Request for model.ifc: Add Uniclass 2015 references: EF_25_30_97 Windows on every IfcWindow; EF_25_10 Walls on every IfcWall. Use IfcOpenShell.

First a look at what the model holds.

```python
import ifcopenshell

model = ifcopenshell.open("model.ifc")
print(model.schema)
print("classifications:", [c.Name for c in model.by_type("IfcClassification")])
for ifc_class in ("IfcDoor", "IfcRoof", "IfcStair", "IfcWall", "IfcWindow"):
    print(ifc_class, len(model.by_type(ifc_class)))
```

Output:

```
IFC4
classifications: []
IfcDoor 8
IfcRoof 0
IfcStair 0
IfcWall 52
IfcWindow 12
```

```python
import ifcopenshell
import ifcopenshell.api.classification

model = ifcopenshell.open("model.ifc")

system = ifcopenshell.api.classification.add_classification(model, classification="Uniclass 2015")

codes = {
    "IfcWindow": ("EF_25_30_97", "Windows"),
    "IfcWall": ("EF_25_10", "Walls"),
}
for ifc_class, (code, name) in codes.items():
    products = model.by_type(ifc_class)
    ifcopenshell.api.classification.add_reference(
        model, products=products, classification=system, identification=code, name=name
    )
    print(code, len(products))

model.write("model_updated.ifc")
```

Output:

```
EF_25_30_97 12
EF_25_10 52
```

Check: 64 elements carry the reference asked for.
